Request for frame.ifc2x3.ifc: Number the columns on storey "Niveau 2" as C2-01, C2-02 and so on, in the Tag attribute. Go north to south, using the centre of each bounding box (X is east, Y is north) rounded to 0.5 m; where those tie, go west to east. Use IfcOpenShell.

First a look at what the model holds.

```python
import ifcopenshell
import ifcopenshell.util.element
import ifcopenshell.util.placement

model = ifcopenshell.open("frame.ifc2x3.ifc")
print(model.schema)
storey = next(s for s in model.by_type("IfcBuildingStorey") if s.Name == "Niveau 2")
columns = [e for e in ifcopenshell.util.element.get_decomposition(storey) if e.is_a("IfcColumn")]
for e in sorted(columns, key=lambda e: e.id()):
    origin = ifcopenshell.util.placement.get_local_placement(e.ObjectPlacement)[:3, 3]
    print(e.id(), e.Tag, e.Name, origin.round(2) + 0.0, sep=" | ")
```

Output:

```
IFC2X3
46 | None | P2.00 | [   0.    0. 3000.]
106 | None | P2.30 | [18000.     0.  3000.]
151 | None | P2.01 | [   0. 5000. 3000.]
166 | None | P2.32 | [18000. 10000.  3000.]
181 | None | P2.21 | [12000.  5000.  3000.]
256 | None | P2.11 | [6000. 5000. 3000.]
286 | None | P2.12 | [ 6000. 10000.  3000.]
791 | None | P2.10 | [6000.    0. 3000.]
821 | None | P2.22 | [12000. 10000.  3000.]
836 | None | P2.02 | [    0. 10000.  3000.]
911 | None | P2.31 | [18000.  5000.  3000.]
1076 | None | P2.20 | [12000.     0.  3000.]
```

```python
import ifcopenshell
import ifcopenshell.geom
import ifcopenshell.util.element
import ifcopenshell.util.shape

model = ifcopenshell.open("frame.ifc2x3.ifc")
settings = ifcopenshell.geom.settings()
settings.set("use-world-coords", True)


def centre(element):
    shape = ifcopenshell.geom.create_shape(settings, element)
    return ifcopenshell.util.shape.get_bbox_centroid(shape.geometry)


storey = next(s for s in model.by_type("IfcBuildingStorey") if s.Name == "Niveau 2")
columns = [e for e in ifcopenshell.util.element.get_decomposition(storey) if e.is_a("IfcColumn")]

# Insertion points can sit at a corner or the storey origin, so sort by the geometry (in metres).
centres = {e: centre(e) for e in columns}
columns.sort(key=lambda e: (-round(centres[e][1] / 0.5), centres[e][0]))

for i, e in enumerate(columns, start=1):
    number = f"C2-{i:02d}"
    e.Tag = number
    print(e.id(), number)

model.write("frame.ifc2x3_updated.ifc")
```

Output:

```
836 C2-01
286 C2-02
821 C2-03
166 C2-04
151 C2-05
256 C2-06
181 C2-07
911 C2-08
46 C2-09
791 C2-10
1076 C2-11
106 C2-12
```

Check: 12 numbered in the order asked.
